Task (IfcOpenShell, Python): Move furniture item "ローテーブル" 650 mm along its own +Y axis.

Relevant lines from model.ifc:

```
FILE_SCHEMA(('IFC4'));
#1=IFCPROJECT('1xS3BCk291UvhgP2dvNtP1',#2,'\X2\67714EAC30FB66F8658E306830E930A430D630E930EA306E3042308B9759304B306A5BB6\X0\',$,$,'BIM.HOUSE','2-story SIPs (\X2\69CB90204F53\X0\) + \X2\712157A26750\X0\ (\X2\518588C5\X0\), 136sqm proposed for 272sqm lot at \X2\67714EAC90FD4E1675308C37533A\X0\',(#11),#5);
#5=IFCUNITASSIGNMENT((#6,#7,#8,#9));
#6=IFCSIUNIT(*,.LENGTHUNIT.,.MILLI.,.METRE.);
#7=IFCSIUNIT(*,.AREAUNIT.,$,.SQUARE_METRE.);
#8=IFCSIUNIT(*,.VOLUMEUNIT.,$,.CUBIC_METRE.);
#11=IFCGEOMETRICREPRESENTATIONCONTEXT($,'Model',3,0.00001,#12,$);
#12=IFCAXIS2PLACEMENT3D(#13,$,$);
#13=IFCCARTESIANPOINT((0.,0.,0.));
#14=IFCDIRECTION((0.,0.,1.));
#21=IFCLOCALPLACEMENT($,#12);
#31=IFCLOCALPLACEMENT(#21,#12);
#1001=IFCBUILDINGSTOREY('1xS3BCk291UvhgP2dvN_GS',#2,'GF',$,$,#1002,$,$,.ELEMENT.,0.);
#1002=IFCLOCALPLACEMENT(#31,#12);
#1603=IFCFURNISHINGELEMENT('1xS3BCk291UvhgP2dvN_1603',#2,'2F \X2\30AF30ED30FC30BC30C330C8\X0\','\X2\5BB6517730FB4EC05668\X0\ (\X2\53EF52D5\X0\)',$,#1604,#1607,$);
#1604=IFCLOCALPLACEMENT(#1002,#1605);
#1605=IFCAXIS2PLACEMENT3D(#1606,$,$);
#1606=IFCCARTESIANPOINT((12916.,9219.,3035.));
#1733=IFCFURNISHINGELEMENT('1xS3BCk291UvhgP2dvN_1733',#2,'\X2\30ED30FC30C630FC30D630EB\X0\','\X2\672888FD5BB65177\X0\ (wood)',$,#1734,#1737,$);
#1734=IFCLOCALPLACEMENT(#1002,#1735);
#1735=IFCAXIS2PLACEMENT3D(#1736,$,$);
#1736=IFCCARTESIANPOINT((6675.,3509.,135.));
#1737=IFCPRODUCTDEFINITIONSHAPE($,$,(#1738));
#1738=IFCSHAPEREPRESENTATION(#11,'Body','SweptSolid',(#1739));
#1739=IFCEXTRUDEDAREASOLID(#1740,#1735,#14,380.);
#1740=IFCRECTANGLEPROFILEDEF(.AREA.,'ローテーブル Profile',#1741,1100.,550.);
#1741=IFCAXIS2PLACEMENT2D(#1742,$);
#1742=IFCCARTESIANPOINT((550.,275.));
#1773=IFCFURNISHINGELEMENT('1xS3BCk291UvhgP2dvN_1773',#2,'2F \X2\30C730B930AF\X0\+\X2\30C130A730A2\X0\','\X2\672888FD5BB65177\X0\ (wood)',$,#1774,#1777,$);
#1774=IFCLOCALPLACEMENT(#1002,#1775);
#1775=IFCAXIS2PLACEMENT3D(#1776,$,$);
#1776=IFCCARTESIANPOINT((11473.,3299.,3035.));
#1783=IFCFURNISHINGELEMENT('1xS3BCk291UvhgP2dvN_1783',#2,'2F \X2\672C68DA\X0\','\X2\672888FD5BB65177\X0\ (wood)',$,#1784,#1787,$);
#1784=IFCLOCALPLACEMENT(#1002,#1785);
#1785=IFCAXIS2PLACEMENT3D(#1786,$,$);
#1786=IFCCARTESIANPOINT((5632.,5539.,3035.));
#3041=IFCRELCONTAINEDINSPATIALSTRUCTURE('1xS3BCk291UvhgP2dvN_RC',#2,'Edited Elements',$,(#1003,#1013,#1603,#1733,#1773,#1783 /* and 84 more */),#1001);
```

```python
import ifcopenshell
import ifcopenshell.api.geometry
import ifcopenshell.util.placement
import ifcopenshell.util.unit

model = ifcopenshell.open("model.ifc")
unit_scale = ifcopenshell.util.unit.calculate_unit_scale(model)

item = model.by_guid("1xS3BCk291UvhgP2dvN_1733")
matrix = ifcopenshell.util.placement.get_local_placement(item.ObjectPlacement)
matrix[:3, 3] += matrix[:3, 1] * 0.65 / unit_scale
ifcopenshell.api.geometry.edit_object_placement(model, product=item, matrix=matrix, is_si=False)

print(ifcopenshell.util.placement.get_local_placement(item.ObjectPlacement).round(3) + 0.0)

model.write("model_edited.ifc")
```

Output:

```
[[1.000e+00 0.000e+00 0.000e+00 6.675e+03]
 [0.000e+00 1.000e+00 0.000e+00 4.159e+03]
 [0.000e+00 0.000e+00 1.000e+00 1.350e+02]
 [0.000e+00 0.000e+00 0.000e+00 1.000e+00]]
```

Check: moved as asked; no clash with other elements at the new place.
